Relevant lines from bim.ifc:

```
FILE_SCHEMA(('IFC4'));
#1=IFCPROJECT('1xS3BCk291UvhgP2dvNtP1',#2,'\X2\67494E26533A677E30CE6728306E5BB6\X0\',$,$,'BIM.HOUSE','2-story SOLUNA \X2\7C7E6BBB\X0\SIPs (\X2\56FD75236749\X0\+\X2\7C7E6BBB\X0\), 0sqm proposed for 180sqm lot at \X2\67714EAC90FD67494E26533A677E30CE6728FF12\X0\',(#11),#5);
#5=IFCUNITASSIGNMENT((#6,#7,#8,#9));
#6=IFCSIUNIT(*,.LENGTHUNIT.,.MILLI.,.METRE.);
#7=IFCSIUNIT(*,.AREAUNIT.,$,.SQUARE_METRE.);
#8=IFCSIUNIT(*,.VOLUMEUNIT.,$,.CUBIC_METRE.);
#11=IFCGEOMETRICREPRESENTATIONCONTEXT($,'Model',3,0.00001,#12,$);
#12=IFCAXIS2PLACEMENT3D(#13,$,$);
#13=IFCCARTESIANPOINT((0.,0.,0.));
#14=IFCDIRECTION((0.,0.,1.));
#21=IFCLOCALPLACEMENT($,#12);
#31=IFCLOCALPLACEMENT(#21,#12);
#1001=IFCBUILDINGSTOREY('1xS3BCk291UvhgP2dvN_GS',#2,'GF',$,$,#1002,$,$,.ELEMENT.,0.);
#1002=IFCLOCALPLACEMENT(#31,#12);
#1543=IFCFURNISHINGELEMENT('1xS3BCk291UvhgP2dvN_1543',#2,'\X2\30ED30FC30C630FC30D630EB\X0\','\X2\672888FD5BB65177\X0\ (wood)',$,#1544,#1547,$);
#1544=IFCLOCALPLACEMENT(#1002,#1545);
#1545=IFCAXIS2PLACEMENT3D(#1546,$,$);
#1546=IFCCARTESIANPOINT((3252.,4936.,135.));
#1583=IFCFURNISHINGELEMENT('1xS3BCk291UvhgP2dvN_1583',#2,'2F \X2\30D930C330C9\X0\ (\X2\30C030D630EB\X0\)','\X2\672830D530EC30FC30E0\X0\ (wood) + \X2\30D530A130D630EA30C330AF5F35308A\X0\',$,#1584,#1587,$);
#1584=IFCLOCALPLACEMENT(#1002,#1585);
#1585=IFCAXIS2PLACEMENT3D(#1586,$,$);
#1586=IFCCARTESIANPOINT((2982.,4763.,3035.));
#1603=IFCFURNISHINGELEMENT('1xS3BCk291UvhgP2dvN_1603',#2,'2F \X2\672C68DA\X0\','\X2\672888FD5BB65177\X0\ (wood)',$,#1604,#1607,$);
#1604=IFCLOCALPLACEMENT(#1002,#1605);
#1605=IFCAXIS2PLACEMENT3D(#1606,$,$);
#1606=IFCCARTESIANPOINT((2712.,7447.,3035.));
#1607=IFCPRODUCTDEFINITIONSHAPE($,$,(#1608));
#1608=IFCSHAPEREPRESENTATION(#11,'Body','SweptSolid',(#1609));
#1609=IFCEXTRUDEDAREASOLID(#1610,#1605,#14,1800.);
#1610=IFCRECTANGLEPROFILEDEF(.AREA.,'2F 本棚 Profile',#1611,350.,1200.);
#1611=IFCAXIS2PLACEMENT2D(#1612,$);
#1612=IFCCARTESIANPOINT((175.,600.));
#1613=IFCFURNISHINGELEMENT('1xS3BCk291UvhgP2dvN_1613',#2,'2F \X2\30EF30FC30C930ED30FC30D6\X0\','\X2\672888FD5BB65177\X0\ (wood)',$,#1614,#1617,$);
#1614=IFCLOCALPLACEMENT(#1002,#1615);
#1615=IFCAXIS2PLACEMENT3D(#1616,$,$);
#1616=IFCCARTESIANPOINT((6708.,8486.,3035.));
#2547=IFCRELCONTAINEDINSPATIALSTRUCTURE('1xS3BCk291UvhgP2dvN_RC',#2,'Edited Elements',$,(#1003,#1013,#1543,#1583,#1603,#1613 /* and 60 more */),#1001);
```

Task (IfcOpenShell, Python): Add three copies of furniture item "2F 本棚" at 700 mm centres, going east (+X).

```python
import numpy as np
import ifcopenshell
import ifcopenshell.api.geometry
import ifcopenshell.api.root
import ifcopenshell.util.element
import ifcopenshell.util.placement

model = ifcopenshell.open("bim.ifc")


def reuse_history(source, copy):
    """copy_class also copies each property set's owner history, people and application; keep the originals."""
    for rel in copy.IsDefinedBy:
        if rel.is_a("IfcRelDefinesByProperties") and (history := rel.RelatingPropertyDefinition.OwnerHistory):
            rel.RelatingPropertyDefinition.OwnerHistory = source.OwnerHistory
            ifcopenshell.util.element.remove_deep2(model, history)


source = model.by_guid("1xS3BCk291UvhgP2dvN_1603")
base = ifcopenshell.util.placement.get_local_placement(source.ObjectPlacement)
step = np.array([1.0, 0.0, 0.0]) * 700.0

for i in range(1, 4):
    copy = ifcopenshell.api.root.copy_class(model, product=source)
    copy.Representation = ifcopenshell.util.element.copy_deep(
        model, source.Representation, exclude=["IfcGeometricRepresentationContext", "IfcRepresentationMap"]
    )
    reuse_history(source, copy)
    matrix = base.copy()
    matrix[:3, 3] += i * step
    print("added at", matrix[:3, 3].round(3) + 0.0)
    ifcopenshell.api.geometry.edit_object_placement(model, product=copy, matrix=matrix, is_si=False)

model.write("bim_rev.ifc")
```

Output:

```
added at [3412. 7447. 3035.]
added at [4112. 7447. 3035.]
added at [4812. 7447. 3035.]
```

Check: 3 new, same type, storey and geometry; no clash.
